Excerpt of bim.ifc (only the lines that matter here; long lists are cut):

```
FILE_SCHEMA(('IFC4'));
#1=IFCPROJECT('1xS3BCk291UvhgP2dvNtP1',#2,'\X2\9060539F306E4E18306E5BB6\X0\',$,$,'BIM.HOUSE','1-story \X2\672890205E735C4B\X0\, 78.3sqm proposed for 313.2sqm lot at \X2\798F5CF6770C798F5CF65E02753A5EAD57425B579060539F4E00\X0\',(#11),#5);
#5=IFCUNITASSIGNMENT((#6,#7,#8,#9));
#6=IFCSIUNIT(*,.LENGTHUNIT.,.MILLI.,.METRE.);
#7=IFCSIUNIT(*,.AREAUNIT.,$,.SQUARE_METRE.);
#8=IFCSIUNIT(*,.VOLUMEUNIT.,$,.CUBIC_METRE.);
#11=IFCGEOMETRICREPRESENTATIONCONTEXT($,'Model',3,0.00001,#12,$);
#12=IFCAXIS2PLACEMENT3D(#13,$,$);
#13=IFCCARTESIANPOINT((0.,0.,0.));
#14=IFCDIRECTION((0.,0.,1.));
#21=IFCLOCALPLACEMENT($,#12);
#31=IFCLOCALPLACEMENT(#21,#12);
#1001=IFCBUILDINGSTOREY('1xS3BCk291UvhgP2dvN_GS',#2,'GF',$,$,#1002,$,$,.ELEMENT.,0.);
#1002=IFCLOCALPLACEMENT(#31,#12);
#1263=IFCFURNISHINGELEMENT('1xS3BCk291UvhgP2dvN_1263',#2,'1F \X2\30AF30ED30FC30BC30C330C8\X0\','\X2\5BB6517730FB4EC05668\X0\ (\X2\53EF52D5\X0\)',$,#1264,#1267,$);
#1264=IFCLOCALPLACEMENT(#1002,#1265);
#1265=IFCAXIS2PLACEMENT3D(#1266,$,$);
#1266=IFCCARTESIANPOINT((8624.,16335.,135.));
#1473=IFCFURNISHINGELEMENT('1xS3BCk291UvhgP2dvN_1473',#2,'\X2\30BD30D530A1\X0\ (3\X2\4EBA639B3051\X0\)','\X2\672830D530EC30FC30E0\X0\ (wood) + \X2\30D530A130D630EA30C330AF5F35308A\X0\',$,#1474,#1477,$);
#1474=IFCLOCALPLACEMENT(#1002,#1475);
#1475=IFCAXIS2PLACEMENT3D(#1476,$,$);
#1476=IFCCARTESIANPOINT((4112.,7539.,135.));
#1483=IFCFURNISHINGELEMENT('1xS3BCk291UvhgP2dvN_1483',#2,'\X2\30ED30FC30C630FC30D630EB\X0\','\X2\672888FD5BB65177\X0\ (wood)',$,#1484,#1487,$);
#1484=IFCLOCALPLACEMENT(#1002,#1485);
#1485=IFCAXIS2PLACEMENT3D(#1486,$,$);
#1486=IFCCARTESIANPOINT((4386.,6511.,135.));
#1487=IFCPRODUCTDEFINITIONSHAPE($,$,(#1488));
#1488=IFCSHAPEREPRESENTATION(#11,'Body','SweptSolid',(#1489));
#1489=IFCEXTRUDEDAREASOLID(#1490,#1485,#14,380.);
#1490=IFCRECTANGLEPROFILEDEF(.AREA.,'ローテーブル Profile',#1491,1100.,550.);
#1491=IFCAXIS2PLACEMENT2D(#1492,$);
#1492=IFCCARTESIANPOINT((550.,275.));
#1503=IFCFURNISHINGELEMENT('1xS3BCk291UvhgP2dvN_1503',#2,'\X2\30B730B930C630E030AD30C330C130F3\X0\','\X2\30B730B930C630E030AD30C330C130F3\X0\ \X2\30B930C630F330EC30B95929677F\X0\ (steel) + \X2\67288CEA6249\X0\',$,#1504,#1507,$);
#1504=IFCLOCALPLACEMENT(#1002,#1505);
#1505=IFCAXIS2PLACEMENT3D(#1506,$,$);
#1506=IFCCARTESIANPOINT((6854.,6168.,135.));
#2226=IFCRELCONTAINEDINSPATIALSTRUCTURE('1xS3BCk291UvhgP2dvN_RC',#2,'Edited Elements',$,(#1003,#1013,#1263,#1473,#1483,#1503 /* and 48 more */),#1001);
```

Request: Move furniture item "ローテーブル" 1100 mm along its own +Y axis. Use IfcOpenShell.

```python
import ifcopenshell
import ifcopenshell.api.geometry
import ifcopenshell.util.placement
import ifcopenshell.util.unit

model = ifcopenshell.open("bim.ifc")
unit_scale = ifcopenshell.util.unit.calculate_unit_scale(model)

item = model.by_guid("1xS3BCk291UvhgP2dvN_1483")
matrix = ifcopenshell.util.placement.get_local_placement(item.ObjectPlacement)
matrix[:3, 3] += matrix[:3, 1] * 1.1 / unit_scale
ifcopenshell.api.geometry.edit_object_placement(model, product=item, matrix=matrix, is_si=False)

print(ifcopenshell.util.placement.get_local_placement(item.ObjectPlacement).round(3) + 0.0)

model.write("bim_edited.ifc")
```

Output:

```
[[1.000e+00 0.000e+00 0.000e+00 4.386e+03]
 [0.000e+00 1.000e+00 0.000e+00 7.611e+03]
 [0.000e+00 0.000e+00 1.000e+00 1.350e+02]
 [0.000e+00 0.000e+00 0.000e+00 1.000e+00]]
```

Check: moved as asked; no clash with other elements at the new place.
